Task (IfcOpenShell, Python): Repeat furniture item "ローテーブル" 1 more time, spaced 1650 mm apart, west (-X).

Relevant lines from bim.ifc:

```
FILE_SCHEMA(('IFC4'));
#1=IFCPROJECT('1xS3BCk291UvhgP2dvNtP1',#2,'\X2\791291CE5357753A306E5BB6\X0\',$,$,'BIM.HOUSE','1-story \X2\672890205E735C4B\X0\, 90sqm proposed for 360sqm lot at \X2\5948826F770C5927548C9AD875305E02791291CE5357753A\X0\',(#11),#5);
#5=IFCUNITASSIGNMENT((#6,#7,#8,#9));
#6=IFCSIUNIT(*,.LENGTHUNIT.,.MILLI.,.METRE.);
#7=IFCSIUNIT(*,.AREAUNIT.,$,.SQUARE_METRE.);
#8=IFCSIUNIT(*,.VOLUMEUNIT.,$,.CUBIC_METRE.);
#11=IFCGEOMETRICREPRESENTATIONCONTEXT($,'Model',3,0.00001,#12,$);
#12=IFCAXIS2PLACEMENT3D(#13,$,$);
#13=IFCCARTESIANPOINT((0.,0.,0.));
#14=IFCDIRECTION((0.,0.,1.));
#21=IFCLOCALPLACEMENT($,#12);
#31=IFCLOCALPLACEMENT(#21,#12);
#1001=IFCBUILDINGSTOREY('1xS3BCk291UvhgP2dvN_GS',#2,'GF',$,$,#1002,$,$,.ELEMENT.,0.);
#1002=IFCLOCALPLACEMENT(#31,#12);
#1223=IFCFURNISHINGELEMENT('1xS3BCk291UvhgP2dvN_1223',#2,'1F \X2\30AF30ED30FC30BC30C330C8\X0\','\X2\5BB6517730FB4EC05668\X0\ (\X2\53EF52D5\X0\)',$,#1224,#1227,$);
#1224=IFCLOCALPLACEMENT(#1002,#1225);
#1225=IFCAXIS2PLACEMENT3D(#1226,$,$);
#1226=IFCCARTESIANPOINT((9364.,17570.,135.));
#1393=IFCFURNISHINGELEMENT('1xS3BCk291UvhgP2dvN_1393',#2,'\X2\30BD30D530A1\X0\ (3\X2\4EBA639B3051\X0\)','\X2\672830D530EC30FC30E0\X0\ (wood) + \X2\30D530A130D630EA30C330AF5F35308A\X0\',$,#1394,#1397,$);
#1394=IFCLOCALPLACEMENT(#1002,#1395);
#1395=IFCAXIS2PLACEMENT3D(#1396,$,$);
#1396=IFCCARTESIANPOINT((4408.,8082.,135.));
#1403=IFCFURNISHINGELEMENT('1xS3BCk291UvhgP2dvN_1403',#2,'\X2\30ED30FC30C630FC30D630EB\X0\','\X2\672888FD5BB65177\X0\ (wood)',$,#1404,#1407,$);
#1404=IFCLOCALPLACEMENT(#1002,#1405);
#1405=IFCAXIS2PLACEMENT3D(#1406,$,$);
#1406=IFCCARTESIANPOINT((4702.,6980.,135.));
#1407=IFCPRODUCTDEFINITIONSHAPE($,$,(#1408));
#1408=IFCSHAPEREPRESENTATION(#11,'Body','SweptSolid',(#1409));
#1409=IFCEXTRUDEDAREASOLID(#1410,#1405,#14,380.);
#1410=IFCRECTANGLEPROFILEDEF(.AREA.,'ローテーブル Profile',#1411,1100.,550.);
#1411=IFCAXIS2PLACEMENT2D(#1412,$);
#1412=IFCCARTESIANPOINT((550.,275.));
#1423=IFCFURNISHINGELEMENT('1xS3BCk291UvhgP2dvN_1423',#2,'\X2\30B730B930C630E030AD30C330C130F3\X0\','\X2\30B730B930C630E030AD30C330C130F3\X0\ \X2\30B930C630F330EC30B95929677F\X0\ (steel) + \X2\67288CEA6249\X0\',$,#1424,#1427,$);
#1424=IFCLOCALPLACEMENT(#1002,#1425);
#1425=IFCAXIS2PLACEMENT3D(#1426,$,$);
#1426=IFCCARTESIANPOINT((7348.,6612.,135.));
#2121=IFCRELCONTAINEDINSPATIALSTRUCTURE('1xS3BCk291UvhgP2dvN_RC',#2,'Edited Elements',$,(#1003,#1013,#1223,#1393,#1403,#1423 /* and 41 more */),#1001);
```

```python
import numpy as np
import ifcopenshell
import ifcopenshell.api.geometry
import ifcopenshell.api.root
import ifcopenshell.util.element
import ifcopenshell.util.placement

model = ifcopenshell.open("bim.ifc")


def reuse_history(source, copy):
    """copy_class also copies each property set's owner history, people and application; keep the originals."""
    for rel in copy.IsDefinedBy:
        if rel.is_a("IfcRelDefinesByProperties") and (history := rel.RelatingPropertyDefinition.OwnerHistory):
            rel.RelatingPropertyDefinition.OwnerHistory = source.OwnerHistory
            ifcopenshell.util.element.remove_deep2(model, history)


source = model.by_id(1403)
base = ifcopenshell.util.placement.get_local_placement(source.ObjectPlacement)
step = np.array([-1.0, 0.0, 0.0]) * 1650.0

for i in range(1, 2):
    copy = ifcopenshell.api.root.copy_class(model, product=source)
    copy.Representation = ifcopenshell.util.element.copy_deep(
        model, source.Representation, exclude=["IfcGeometricRepresentationContext", "IfcRepresentationMap"]
    )
    reuse_history(source, copy)
    matrix = base.copy()
    matrix[:3, 3] += i * step
    print("added at", matrix[:3, 3].round(3) + 0.0)
    ifcopenshell.api.geometry.edit_object_placement(model, product=copy, matrix=matrix, is_si=False)

model.write("bim_edited.ifc")
```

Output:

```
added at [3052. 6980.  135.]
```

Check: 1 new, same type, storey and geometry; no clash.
